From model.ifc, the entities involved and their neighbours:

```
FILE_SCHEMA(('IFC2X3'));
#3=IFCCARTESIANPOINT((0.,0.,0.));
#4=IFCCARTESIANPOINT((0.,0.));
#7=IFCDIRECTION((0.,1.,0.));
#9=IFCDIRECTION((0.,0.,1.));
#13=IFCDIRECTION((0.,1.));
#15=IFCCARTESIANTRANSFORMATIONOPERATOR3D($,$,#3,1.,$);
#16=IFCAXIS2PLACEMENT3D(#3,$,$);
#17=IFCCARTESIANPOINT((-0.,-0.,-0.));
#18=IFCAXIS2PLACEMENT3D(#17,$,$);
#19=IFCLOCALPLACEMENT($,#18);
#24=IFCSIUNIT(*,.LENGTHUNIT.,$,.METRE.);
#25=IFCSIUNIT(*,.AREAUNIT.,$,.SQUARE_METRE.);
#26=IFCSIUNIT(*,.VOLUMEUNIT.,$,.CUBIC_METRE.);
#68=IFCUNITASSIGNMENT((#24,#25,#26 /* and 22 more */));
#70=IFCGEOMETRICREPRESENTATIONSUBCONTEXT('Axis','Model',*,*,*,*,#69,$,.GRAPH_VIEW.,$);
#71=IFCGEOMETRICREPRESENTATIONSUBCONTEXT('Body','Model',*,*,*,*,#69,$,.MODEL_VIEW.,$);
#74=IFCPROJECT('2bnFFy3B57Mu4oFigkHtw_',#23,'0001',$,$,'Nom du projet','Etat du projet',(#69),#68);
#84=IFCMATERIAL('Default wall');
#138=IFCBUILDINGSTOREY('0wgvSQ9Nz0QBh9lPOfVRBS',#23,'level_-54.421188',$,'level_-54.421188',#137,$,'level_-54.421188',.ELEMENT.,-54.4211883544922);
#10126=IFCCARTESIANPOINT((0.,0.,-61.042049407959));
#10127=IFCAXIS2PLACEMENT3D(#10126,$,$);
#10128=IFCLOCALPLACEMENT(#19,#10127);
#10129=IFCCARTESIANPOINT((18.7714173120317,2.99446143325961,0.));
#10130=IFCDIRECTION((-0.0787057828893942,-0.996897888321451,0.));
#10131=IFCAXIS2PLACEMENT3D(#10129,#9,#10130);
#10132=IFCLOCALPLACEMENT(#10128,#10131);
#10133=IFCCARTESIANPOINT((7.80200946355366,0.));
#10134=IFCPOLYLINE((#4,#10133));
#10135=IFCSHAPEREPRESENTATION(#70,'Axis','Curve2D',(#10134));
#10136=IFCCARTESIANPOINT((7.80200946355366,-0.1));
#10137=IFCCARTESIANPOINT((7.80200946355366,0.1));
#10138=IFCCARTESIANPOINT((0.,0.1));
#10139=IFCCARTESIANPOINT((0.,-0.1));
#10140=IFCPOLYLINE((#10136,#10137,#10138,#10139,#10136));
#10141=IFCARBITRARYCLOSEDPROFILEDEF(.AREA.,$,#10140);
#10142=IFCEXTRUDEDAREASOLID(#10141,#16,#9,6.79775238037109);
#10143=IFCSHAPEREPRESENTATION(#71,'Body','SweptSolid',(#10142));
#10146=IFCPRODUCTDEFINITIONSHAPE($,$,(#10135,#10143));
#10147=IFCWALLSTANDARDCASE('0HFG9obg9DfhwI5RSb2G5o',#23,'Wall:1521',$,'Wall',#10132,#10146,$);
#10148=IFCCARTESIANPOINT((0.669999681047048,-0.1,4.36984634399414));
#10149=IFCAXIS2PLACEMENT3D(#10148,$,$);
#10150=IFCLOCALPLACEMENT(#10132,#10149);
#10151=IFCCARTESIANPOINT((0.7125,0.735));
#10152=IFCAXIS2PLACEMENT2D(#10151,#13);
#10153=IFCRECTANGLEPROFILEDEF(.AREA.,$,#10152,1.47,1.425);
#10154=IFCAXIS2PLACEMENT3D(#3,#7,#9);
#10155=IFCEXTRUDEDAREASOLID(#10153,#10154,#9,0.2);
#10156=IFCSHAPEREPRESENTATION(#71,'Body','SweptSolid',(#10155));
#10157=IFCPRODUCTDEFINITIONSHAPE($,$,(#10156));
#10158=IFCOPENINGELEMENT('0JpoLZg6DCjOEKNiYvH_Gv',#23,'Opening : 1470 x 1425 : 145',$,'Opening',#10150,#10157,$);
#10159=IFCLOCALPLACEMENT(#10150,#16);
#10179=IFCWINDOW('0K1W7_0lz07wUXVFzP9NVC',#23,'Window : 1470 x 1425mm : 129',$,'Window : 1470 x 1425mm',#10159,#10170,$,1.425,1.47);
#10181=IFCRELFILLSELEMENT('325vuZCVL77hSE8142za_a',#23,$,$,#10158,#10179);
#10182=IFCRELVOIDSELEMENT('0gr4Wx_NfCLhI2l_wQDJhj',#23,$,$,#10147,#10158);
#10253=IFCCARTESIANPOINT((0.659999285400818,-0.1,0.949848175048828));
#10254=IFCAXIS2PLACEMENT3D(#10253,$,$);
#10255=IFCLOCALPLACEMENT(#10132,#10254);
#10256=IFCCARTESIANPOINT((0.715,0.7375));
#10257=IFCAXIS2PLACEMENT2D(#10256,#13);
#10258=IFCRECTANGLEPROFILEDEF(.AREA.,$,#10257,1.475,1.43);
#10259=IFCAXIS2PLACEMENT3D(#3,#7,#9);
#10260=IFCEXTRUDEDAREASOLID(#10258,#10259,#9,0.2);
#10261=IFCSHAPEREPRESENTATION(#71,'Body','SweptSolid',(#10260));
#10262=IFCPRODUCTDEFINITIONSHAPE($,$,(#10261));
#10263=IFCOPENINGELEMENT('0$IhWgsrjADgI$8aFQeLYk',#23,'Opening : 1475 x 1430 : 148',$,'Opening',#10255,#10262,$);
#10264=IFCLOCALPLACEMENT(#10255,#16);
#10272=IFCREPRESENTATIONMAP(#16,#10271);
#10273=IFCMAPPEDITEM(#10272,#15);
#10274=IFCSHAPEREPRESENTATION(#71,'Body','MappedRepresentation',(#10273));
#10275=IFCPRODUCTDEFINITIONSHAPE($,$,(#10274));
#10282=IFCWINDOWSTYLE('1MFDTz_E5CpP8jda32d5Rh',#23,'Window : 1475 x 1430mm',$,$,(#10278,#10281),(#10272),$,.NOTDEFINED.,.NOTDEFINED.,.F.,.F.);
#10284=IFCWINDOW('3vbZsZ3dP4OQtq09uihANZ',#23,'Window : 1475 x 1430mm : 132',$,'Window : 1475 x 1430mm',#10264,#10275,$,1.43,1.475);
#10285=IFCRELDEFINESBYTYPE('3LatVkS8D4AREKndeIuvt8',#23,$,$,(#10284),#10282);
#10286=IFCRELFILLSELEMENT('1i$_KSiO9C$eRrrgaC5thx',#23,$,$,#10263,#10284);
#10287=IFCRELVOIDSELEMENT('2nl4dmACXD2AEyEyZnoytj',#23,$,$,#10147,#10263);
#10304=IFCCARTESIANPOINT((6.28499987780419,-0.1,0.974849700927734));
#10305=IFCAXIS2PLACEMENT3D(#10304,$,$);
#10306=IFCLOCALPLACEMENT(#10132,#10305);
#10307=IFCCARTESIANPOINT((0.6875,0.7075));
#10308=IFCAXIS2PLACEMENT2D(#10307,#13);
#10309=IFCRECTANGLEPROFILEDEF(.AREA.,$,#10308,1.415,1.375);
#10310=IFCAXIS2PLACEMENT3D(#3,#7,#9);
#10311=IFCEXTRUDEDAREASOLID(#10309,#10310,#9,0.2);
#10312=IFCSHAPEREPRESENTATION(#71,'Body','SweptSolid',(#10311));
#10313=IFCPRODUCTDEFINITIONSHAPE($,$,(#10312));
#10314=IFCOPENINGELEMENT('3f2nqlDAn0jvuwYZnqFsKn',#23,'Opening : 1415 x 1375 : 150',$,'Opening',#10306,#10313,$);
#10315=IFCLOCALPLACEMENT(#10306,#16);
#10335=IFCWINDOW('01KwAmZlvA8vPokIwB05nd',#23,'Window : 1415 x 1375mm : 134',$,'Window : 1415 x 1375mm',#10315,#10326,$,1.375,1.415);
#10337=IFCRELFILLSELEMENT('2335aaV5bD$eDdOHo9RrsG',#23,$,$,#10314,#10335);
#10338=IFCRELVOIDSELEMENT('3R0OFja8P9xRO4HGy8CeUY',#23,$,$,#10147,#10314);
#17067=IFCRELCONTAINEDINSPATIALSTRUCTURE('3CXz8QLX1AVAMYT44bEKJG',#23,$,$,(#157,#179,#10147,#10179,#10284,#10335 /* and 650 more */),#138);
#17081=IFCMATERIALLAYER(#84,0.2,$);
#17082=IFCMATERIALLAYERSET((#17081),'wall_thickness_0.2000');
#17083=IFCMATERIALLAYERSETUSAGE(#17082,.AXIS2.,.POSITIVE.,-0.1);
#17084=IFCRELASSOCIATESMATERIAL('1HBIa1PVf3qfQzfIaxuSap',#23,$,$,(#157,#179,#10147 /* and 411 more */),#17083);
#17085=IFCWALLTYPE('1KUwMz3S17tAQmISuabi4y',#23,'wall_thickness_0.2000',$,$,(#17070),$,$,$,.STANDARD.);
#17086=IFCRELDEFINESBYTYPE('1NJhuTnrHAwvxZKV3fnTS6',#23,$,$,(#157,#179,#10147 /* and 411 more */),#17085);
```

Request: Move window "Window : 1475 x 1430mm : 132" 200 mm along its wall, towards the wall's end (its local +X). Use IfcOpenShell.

```python
import ifcopenshell
import ifcopenshell.api.geometry
import ifcopenshell.util.placement

model = ifcopenshell.open("model.ifc")

window = model.by_guid("3vbZsZ3dP4OQtq09uihANZ")
opening = window.FillsVoids[0].RelatingOpeningElement
wall = opening.VoidsElements[0].RelatingBuildingElement

wall_matrix = ifcopenshell.util.placement.get_local_placement(wall.ObjectPlacement)
shift = wall_matrix[:3, 0] * 0.2
before = ifcopenshell.util.placement.get_local_placement(window.ObjectPlacement)[:3, 3].copy()

# The window is placed relative to its opening, so it follows when the opening moves.
matrix = ifcopenshell.util.placement.get_local_placement(opening.ObjectPlacement)
matrix[:3, 3] += shift
ifcopenshell.api.geometry.edit_object_placement(
    model, product=opening, matrix=matrix, is_si=False, should_transform_children=True
)

after = ifcopenshell.util.placement.get_local_placement(window.ObjectPlacement)[:3, 3]
print("window moved by", (after - before).round(3) + 0.0)

model.write("model_rev.ifc")
```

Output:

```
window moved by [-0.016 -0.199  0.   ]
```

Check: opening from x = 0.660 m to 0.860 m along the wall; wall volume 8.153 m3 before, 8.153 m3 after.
